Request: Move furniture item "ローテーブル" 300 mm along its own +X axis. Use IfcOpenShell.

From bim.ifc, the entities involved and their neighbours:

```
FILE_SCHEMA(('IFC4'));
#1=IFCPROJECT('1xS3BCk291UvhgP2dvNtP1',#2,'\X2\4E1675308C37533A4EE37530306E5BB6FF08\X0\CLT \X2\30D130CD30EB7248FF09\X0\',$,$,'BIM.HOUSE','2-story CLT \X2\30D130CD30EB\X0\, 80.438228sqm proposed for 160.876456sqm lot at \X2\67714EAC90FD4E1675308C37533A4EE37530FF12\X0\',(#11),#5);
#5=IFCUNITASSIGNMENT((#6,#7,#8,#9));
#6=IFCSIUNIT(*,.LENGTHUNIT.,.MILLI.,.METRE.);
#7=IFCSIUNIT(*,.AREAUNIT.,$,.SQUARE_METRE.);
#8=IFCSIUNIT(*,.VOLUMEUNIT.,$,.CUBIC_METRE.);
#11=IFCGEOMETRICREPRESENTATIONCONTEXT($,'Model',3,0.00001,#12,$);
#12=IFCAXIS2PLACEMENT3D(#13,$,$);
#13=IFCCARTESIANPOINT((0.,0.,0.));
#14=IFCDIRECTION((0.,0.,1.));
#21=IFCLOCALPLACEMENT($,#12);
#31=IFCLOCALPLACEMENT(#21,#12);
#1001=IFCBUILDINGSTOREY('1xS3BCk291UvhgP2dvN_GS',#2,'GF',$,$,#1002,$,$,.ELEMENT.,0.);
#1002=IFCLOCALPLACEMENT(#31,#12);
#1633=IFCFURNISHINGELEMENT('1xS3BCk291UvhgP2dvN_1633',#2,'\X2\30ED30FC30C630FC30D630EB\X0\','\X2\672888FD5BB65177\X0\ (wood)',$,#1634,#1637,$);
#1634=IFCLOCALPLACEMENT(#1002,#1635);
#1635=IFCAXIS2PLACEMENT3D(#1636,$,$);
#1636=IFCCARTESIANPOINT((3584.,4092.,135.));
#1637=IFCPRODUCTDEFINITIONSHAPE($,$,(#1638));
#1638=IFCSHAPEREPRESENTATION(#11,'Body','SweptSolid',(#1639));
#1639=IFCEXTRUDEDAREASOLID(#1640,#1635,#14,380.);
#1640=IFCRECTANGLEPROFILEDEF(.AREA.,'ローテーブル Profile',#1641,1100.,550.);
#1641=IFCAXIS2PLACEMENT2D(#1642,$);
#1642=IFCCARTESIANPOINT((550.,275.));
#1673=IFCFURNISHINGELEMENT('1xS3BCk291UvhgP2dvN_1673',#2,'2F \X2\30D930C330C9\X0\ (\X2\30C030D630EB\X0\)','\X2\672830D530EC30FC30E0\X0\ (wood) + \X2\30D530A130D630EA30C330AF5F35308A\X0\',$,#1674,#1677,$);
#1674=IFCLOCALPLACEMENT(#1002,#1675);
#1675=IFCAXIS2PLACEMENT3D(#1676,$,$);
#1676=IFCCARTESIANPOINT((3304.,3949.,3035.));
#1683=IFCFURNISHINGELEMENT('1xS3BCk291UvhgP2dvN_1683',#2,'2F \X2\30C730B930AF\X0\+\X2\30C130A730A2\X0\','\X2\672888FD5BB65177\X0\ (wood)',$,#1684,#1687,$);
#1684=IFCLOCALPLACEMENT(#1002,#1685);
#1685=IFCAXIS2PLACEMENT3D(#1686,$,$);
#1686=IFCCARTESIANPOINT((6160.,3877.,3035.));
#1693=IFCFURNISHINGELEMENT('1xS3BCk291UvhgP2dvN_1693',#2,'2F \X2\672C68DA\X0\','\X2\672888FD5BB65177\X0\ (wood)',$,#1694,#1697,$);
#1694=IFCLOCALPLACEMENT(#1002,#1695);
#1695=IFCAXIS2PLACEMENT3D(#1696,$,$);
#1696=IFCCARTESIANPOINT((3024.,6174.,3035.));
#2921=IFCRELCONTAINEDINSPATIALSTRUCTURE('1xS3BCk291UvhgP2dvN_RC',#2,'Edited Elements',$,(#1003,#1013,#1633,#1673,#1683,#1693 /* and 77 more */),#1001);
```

```python
import ifcopenshell
import ifcopenshell.api.geometry
import ifcopenshell.util.placement

model = ifcopenshell.open("bim.ifc")

item = model.by_guid("1xS3BCk291UvhgP2dvN_1633")
matrix = ifcopenshell.util.placement.get_local_placement(item.ObjectPlacement)
matrix[:3, 3] += matrix[:3, 0] * 300.0
ifcopenshell.api.geometry.edit_object_placement(model, product=item, matrix=matrix, is_si=False)

print(ifcopenshell.util.placement.get_local_placement(item.ObjectPlacement).round(3) + 0.0)

model.write("bim_v2.ifc")
```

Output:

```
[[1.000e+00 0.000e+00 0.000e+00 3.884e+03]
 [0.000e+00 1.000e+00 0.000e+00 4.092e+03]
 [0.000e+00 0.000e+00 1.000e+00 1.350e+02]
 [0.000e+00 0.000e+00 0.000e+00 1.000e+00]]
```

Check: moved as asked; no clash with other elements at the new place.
